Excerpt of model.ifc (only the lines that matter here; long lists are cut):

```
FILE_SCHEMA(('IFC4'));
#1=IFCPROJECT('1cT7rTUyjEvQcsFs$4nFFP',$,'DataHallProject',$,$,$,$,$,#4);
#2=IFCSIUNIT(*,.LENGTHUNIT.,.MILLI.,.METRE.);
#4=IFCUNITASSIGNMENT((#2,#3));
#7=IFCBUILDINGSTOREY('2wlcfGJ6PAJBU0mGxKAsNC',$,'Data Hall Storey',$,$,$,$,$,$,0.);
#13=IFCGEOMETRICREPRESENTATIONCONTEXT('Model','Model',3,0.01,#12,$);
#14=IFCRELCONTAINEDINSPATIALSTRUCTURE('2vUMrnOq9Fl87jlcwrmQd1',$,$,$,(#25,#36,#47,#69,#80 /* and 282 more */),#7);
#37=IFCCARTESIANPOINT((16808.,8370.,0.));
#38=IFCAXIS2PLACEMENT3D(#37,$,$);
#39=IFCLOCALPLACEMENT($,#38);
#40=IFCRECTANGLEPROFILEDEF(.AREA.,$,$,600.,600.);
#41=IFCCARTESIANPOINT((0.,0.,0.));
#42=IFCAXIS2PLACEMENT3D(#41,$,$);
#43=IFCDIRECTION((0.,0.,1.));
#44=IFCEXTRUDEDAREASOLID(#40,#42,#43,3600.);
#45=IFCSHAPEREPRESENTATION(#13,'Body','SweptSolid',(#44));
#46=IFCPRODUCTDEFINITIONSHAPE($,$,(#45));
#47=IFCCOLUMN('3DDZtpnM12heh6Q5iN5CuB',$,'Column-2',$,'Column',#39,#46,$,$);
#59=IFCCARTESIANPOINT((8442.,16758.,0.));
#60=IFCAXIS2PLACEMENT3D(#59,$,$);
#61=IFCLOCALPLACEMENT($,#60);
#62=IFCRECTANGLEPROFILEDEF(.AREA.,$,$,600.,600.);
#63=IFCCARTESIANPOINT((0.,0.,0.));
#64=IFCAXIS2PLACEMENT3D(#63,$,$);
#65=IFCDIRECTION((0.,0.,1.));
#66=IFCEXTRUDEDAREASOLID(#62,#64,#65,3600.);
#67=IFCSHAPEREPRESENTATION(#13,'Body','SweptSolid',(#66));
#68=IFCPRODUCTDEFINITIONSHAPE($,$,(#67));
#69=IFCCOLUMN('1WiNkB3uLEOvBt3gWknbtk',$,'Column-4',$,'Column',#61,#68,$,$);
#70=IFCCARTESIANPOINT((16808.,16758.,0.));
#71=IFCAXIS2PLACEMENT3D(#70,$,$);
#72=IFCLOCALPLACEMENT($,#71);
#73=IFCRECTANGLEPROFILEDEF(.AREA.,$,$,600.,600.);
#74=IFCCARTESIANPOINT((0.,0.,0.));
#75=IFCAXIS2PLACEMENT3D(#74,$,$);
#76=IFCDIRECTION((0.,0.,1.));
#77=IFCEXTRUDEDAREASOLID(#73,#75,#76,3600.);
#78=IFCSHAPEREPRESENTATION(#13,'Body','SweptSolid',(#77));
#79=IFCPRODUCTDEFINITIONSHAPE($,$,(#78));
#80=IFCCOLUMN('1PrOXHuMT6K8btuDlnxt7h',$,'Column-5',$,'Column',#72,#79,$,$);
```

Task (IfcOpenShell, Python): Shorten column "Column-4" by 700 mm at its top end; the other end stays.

```python
import ifcopenshell
import ifcopenshell.util.unit

model = ifcopenshell.open("model.ifc")
unit_scale = ifcopenshell.util.unit.calculate_unit_scale(model)

member = model.by_guid("1WiNkB3uLEOvBt3gWknbtk")
change = -0.7 / unit_scale

# The extrusion runs towards the end named, so only its depth changes.
body = next(r for r in member.Representation.Representations if r.RepresentationIdentifier == "Body")
solid = body.Items[0]
old_length = solid.Depth
solid.Depth += change

print(f"length {old_length:g} -> {solid.Depth:g}")

model.write("model_rev.ifc")
```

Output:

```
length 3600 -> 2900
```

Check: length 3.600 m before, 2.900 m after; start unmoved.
